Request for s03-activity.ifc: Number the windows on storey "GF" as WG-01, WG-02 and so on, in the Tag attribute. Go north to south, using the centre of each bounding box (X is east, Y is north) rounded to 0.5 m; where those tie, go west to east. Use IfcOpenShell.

First a look at what the model holds.

```python
import ifcopenshell
import ifcopenshell.util.element
import ifcopenshell.util.placement

model = ifcopenshell.open("s03-activity.ifc")
print(model.schema)
storey = next(s for s in model.by_type("IfcBuildingStorey") if s.Name == "GF")
windows = [e for e in ifcopenshell.util.element.get_decomposition(storey) if e.is_a("IfcWindow")]
for e in sorted(windows, key=lambda e: e.id()):
    origin = ifcopenshell.util.placement.get_local_placement(e.ObjectPlacement)[:3, 3]
    print(e.id(), e.Tag, e.Name, origin.round(2) + 0.0, sep=" | ")
```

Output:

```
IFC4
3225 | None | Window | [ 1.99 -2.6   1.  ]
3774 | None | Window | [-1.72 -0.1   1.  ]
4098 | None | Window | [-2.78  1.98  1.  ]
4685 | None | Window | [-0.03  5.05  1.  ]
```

```python
import ifcopenshell
import ifcopenshell.geom
import ifcopenshell.util.element
import ifcopenshell.util.shape

model = ifcopenshell.open("s03-activity.ifc")
settings = ifcopenshell.geom.settings()
settings.set("use-world-coords", True)


def centre(element):
    shape = ifcopenshell.geom.create_shape(settings, element)
    return ifcopenshell.util.shape.get_bbox_centroid(shape.geometry)


storey = next(s for s in model.by_type("IfcBuildingStorey") if s.Name == "GF")
windows = [e for e in ifcopenshell.util.element.get_decomposition(storey) if e.is_a("IfcWindow")]

# Insertion points can sit at a corner or the storey origin, so sort by the geometry (in metres).
centres = {e: centre(e) for e in windows}
windows.sort(key=lambda e: (-round(centres[e][1] / 0.5), centres[e][0]))

for i, e in enumerate(windows, start=1):
    number = f"WG-{i:02d}"
    e.Tag = number
    print(e.id(), number)

model.write("s03-activity-out.ifc")
```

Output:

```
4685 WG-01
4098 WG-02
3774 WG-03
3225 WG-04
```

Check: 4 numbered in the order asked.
